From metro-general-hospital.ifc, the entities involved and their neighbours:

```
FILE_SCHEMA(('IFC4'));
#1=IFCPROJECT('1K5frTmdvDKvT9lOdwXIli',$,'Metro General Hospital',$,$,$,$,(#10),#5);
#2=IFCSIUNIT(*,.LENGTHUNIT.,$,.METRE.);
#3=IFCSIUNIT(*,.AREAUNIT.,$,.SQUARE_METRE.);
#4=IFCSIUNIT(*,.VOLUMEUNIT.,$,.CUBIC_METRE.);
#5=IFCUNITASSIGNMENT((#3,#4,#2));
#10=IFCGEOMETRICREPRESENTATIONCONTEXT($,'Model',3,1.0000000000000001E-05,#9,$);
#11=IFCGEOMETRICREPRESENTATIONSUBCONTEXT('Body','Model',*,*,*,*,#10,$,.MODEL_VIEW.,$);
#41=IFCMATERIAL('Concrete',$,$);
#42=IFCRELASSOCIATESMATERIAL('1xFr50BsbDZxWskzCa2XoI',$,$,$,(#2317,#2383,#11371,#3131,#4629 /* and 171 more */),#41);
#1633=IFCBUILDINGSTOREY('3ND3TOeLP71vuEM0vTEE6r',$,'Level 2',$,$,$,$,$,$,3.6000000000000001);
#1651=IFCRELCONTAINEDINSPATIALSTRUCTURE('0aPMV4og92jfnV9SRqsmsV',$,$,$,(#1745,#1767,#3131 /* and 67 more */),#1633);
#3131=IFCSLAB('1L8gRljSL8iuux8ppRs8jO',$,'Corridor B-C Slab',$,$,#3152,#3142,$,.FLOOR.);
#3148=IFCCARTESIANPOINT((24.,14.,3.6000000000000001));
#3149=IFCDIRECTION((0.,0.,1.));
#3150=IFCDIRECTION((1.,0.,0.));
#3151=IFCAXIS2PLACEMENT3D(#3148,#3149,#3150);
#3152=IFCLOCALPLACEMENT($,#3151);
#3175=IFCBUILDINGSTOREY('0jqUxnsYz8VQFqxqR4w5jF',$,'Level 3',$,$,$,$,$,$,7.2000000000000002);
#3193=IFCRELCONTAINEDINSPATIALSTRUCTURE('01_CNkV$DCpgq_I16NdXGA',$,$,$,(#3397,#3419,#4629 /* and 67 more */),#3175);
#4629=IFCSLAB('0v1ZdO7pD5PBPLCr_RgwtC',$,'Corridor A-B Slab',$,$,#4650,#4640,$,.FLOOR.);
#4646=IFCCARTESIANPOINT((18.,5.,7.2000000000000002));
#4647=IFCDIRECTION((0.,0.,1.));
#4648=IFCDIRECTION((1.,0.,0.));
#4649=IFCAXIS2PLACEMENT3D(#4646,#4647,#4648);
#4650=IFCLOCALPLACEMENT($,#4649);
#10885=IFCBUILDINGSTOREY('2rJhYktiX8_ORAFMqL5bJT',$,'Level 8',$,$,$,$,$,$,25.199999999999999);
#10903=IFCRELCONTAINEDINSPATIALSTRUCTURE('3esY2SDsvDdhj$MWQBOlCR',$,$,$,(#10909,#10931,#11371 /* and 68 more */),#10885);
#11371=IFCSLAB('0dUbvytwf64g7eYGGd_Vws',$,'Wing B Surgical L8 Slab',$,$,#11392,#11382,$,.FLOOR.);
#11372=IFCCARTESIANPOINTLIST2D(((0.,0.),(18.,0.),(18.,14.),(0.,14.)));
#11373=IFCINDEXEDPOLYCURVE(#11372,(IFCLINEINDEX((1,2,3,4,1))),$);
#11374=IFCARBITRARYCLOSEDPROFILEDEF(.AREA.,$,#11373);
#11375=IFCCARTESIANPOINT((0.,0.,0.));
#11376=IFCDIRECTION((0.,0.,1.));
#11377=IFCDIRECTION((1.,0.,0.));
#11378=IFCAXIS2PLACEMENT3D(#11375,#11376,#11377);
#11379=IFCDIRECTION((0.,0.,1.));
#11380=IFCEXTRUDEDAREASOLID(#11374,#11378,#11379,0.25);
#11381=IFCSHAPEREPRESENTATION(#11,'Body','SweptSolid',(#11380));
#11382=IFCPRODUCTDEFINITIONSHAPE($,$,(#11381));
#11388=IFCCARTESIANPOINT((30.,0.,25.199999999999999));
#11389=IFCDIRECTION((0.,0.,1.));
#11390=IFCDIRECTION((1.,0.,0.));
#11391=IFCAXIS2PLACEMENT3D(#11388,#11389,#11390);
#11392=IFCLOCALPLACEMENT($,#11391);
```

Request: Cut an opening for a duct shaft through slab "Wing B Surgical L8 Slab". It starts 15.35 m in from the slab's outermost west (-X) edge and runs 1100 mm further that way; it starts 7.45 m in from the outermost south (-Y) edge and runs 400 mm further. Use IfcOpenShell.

```python
import numpy as np
import ifcopenshell
import ifcopenshell.api.feature
import ifcopenshell.api.geometry
import ifcopenshell.api.root
import ifcopenshell.geom
import ifcopenshell.util.placement
import ifcopenshell.util.representation
import ifcopenshell.util.shape
import ifcopenshell.util.unit

model = ifcopenshell.open("metro-general-hospital.ifc")
unit_scale = ifcopenshell.util.unit.calculate_unit_scale(model)
settings = ifcopenshell.geom.settings()


def volume(element):
    """Net volume in cubic metres, openings subtracted."""
    shape = ifcopenshell.geom.create_shape(settings, element)
    return ifcopenshell.util.shape.get_volume(shape.geometry)


slab = model.by_guid("0dUbvytwf64g7eYGGd_Vws")
before = volume(slab)

# Extent in the slab's own axes, in metres. The edges named are its -X and -Y sides.
slab_shape = ifcopenshell.geom.create_shape(settings, slab)
vertices = ifcopenshell.util.shape.get_vertices(slab_shape.geometry)
x_min, y_min, bottom = vertices.min(axis=0)
top = vertices[:, 2].max()

opening = ifcopenshell.api.root.create_entity(model, ifc_class="IfcOpeningElement", name="Duct shaft opening", predefined_type="OPENING")
context = ifcopenshell.util.representation.get_context(model, "Model", "Body", "MODEL_VIEW")
width, depth = 1.1, 0.4
outline = [(0.0, 0.0), (width, 0.0), (width, depth), (0.0, depth), (0.0, 0.0)]
# Overshoot both faces by 50 mm so the cut is clean.
shape = ifcopenshell.api.geometry.add_slab_representation(
    model, context=context, depth=top - bottom + 0.1, polyline=outline
)
ifcopenshell.api.geometry.assign_representation(model, product=opening, representation=shape)

matrix = ifcopenshell.util.placement.get_local_placement(slab.ObjectPlacement)
matrix[:, 3] = matrix @ np.append(np.array([x_min + 15.35, y_min + 7.45, bottom - 0.05]) / unit_scale, 1.0)
ifcopenshell.api.geometry.edit_object_placement(model, product=opening, matrix=matrix, is_si=False)
ifcopenshell.api.feature.add_feature(model, feature=opening, element=slab)

after = volume(slab)

print(f"slab volume {before:.3f} -> {after:.3f} m3")

model.write("metro-general-hospital-out.ifc")
```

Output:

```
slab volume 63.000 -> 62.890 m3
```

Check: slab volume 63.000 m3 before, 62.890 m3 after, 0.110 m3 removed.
